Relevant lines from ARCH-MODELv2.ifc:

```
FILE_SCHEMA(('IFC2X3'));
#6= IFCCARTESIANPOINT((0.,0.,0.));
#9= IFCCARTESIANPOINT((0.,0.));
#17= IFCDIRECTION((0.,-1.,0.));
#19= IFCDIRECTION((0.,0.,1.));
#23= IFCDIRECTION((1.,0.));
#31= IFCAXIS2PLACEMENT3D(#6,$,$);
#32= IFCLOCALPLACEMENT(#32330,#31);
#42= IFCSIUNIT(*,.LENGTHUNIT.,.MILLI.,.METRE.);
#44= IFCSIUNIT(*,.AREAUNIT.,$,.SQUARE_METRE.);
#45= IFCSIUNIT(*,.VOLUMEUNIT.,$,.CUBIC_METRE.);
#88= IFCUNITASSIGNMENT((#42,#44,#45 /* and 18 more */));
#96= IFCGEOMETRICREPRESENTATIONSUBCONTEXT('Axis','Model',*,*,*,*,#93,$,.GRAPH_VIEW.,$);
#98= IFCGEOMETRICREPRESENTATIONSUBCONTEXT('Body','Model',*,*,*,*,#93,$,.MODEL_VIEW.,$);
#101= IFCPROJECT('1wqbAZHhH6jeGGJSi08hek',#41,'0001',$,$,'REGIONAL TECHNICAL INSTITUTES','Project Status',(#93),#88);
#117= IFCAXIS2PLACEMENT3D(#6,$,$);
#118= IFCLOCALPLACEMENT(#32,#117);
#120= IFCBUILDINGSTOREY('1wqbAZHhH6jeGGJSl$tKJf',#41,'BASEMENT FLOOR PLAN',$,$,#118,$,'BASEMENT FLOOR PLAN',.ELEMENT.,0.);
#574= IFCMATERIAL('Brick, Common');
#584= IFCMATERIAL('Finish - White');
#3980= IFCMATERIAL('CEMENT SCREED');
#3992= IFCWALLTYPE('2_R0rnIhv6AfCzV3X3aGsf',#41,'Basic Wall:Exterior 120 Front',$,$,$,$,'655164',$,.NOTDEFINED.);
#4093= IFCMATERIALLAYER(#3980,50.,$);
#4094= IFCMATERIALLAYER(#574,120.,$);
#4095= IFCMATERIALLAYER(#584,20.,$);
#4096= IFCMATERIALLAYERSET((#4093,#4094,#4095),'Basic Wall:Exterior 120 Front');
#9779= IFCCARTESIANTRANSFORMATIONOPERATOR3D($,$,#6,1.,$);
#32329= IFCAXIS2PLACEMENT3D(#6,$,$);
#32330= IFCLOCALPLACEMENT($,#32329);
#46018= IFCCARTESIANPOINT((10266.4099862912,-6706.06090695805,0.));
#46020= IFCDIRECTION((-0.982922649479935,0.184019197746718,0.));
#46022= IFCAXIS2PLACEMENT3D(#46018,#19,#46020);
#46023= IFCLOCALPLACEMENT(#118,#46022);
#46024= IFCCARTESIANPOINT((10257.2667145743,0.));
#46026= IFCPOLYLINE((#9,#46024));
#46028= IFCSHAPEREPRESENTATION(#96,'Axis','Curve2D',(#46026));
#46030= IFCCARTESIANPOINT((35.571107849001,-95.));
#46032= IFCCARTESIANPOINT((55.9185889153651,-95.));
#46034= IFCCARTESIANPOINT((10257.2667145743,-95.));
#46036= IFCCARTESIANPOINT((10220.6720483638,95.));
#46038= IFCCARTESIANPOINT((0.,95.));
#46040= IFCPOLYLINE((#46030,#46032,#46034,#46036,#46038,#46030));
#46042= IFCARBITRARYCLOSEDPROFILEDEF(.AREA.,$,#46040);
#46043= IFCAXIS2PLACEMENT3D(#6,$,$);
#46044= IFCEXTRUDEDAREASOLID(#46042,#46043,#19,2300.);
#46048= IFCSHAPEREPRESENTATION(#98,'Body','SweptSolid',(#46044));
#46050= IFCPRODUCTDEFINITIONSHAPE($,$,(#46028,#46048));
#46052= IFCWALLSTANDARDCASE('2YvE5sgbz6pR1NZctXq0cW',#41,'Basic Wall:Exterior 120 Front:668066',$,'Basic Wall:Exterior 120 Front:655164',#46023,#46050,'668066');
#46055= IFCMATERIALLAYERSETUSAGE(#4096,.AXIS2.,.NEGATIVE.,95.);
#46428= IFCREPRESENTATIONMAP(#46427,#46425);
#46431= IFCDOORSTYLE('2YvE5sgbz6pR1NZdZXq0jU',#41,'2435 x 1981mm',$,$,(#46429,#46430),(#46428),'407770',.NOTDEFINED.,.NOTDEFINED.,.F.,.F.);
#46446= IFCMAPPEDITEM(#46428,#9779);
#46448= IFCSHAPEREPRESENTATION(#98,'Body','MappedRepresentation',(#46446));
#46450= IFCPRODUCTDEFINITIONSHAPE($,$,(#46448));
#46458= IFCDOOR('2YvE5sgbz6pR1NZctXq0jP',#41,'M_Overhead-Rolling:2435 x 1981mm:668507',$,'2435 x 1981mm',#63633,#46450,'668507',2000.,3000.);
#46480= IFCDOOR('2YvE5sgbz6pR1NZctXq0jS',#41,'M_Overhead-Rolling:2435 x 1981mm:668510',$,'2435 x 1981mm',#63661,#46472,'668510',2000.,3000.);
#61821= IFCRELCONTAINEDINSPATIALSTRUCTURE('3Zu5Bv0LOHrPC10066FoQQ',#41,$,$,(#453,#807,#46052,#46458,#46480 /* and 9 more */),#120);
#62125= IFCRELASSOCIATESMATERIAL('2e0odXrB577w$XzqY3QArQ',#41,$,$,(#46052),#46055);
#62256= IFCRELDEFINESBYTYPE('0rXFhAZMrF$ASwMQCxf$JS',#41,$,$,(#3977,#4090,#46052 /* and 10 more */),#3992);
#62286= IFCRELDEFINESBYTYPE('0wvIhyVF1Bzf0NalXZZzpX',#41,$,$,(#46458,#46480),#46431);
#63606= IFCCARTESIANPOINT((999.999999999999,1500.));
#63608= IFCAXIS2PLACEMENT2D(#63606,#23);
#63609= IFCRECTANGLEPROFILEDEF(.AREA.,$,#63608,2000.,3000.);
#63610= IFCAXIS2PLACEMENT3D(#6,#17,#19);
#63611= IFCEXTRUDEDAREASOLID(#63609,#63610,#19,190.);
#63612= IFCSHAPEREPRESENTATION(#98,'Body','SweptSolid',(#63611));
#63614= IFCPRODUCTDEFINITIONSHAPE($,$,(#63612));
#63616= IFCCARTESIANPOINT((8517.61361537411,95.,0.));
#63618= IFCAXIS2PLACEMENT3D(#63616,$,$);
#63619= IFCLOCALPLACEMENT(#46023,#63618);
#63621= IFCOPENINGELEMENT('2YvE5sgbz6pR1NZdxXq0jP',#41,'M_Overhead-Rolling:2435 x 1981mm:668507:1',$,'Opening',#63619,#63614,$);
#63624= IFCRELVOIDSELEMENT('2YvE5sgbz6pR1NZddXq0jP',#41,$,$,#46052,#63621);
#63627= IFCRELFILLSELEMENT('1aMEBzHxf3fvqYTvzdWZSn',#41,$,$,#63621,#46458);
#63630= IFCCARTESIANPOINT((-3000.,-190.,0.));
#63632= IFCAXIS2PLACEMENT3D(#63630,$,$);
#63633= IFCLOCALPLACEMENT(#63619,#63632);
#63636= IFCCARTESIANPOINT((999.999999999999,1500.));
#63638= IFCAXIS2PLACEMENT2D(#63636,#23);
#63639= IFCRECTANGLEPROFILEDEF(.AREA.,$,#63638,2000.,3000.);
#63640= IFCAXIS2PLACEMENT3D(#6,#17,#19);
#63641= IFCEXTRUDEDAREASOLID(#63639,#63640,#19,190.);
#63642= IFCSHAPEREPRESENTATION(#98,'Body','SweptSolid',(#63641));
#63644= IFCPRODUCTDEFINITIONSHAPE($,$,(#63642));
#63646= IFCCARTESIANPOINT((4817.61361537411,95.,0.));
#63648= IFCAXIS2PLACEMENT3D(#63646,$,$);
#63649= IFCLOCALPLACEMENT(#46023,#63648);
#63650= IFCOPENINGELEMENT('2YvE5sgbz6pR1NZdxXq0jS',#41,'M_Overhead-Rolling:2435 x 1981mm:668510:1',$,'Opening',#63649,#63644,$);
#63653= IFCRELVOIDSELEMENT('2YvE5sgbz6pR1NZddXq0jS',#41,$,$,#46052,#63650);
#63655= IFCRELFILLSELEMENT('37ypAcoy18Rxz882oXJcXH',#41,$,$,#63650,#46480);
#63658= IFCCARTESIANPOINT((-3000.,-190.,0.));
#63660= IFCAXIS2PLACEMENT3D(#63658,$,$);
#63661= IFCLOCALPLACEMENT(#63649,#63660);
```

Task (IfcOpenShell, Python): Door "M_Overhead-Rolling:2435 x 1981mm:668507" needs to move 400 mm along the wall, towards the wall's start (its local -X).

```python
import ifcopenshell
import ifcopenshell.api.geometry
import ifcopenshell.util.placement

model = ifcopenshell.open("ARCH-MODELv2.ifc")

door = model.by_guid("2YvE5sgbz6pR1NZctXq0jP")
opening = door.FillsVoids[0].RelatingOpeningElement
wall = opening.VoidsElements[0].RelatingBuildingElement

wall_matrix = ifcopenshell.util.placement.get_local_placement(wall.ObjectPlacement)
shift = wall_matrix[:3, 0] * -400.0
before = ifcopenshell.util.placement.get_local_placement(door.ObjectPlacement)[:3, 3].copy()

# The door is placed relative to its opening, so it follows when the opening moves.
matrix = ifcopenshell.util.placement.get_local_placement(opening.ObjectPlacement)
matrix[:3, 3] += shift
ifcopenshell.api.geometry.edit_object_placement(
    model, product=opening, matrix=matrix, is_si=False, should_transform_children=True
)

after = ifcopenshell.util.placement.get_local_placement(door.ObjectPlacement)[:3, 3]
print("door moved by", (after - before).round(3) + 0.0)

model.write("ARCH-MODELv2_updated.ifc")
```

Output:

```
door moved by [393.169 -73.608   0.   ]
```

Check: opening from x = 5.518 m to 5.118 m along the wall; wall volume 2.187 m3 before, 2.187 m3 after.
